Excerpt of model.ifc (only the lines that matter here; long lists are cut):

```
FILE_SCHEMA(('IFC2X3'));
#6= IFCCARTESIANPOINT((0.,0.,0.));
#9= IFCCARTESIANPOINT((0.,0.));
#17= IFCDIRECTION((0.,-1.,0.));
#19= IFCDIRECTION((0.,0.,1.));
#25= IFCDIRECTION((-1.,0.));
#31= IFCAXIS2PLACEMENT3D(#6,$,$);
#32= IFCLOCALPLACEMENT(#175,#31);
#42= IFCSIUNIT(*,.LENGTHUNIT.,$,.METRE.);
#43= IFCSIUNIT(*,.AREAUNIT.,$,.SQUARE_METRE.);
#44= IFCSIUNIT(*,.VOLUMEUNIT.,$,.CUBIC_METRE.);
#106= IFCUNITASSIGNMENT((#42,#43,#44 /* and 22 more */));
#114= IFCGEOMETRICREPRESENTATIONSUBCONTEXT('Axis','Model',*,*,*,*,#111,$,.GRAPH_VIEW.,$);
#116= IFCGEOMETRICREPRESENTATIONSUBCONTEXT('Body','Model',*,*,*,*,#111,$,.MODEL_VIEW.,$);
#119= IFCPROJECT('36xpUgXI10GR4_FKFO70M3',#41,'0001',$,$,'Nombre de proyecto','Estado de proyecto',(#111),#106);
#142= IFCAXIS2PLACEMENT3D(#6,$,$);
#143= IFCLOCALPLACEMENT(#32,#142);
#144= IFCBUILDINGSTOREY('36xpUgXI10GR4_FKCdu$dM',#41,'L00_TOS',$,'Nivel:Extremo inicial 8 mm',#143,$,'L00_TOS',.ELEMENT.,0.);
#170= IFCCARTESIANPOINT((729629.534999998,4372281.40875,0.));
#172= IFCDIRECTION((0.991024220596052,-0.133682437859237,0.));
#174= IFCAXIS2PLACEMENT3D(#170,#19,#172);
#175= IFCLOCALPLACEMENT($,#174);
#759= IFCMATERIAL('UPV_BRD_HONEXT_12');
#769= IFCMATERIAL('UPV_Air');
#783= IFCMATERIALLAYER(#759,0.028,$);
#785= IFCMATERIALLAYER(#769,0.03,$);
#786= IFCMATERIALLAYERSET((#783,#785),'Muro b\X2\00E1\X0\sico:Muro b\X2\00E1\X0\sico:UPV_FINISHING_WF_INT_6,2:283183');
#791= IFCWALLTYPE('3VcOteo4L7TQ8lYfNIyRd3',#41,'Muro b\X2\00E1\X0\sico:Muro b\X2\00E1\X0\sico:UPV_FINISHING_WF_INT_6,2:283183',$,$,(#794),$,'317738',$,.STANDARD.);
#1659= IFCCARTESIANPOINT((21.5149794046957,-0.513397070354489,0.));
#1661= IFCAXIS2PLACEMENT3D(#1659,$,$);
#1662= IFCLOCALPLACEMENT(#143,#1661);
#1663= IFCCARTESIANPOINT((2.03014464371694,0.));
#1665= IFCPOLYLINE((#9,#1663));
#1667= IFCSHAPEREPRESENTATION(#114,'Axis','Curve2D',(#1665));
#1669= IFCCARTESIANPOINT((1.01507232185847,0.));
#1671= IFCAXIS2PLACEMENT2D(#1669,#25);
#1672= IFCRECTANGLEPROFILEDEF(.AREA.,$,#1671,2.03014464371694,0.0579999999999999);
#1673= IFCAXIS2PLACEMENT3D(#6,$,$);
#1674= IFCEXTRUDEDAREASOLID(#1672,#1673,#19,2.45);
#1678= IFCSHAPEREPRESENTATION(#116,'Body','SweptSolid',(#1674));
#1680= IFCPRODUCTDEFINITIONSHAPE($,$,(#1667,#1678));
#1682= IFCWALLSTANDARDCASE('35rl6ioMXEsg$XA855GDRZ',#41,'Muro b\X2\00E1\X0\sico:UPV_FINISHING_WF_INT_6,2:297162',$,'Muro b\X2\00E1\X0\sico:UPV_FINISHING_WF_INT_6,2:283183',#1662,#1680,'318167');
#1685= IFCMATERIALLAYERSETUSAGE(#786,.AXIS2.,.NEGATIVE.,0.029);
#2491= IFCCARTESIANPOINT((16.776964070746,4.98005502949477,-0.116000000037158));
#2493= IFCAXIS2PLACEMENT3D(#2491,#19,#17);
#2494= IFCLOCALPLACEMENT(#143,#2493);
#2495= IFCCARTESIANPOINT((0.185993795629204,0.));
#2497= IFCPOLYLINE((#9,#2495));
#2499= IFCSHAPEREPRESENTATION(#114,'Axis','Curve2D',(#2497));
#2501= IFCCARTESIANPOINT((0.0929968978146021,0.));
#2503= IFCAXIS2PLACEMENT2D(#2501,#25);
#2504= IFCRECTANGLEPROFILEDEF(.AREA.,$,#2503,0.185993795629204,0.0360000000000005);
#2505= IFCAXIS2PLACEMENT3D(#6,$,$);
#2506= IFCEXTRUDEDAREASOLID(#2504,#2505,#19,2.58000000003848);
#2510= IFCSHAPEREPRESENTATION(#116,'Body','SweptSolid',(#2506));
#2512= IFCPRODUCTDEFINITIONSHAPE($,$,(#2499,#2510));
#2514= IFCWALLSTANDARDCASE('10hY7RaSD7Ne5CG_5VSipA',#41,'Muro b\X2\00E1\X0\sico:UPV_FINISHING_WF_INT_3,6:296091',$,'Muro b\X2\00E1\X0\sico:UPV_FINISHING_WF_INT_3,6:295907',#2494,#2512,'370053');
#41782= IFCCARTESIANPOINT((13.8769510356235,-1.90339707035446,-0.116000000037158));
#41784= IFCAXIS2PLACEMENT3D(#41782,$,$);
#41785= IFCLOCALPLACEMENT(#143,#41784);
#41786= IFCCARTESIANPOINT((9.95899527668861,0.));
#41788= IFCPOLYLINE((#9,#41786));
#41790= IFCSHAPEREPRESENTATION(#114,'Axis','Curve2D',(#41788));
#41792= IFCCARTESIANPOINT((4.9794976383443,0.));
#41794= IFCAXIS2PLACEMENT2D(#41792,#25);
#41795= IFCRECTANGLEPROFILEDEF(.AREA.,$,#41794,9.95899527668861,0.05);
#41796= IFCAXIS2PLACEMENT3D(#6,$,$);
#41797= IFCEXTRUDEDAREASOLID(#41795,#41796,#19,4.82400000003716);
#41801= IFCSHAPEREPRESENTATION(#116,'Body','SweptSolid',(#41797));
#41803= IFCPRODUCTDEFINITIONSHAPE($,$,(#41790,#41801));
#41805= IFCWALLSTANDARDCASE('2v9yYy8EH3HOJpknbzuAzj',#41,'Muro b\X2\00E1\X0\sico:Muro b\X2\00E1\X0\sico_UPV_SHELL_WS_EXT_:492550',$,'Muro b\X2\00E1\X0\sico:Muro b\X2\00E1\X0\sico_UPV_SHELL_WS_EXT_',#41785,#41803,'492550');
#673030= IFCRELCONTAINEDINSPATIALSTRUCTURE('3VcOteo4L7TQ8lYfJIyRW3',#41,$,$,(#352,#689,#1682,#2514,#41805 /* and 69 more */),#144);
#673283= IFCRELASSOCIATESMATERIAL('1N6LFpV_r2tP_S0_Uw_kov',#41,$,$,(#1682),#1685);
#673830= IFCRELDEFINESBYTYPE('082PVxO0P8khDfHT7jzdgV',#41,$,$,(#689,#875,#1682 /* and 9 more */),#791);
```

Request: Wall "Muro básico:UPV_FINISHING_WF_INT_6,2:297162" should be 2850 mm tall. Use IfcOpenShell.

```python
import ifcopenshell
import ifcopenshell.geom
import ifcopenshell.util.representation
import ifcopenshell.util.shape
import ifcopenshell.util.unit

model = ifcopenshell.open("model.ifc")
unit_scale = ifcopenshell.util.unit.calculate_unit_scale(model)
settings = ifcopenshell.geom.settings()


def volume(element):
    """Net volume in cubic metres, openings subtracted."""
    shape = ifcopenshell.geom.create_shape(settings, element)
    return ifcopenshell.util.shape.get_volume(shape.geometry)


wall = model.by_id(1682)
before = volume(wall)

body = ifcopenshell.util.representation.get_representation(wall, "Model", "Body")
solid = body.Items[0]
old_height = solid.Depth
solid.Depth = 2.85 / unit_scale
after = volume(wall)

print(f"height {old_height:g} -> {solid.Depth:g}, volume {before:.3f} -> {after:.3f} m3")

model.write("model_v2.ifc")
```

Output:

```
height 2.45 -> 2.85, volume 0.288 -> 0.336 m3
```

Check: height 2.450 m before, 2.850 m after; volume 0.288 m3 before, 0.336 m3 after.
